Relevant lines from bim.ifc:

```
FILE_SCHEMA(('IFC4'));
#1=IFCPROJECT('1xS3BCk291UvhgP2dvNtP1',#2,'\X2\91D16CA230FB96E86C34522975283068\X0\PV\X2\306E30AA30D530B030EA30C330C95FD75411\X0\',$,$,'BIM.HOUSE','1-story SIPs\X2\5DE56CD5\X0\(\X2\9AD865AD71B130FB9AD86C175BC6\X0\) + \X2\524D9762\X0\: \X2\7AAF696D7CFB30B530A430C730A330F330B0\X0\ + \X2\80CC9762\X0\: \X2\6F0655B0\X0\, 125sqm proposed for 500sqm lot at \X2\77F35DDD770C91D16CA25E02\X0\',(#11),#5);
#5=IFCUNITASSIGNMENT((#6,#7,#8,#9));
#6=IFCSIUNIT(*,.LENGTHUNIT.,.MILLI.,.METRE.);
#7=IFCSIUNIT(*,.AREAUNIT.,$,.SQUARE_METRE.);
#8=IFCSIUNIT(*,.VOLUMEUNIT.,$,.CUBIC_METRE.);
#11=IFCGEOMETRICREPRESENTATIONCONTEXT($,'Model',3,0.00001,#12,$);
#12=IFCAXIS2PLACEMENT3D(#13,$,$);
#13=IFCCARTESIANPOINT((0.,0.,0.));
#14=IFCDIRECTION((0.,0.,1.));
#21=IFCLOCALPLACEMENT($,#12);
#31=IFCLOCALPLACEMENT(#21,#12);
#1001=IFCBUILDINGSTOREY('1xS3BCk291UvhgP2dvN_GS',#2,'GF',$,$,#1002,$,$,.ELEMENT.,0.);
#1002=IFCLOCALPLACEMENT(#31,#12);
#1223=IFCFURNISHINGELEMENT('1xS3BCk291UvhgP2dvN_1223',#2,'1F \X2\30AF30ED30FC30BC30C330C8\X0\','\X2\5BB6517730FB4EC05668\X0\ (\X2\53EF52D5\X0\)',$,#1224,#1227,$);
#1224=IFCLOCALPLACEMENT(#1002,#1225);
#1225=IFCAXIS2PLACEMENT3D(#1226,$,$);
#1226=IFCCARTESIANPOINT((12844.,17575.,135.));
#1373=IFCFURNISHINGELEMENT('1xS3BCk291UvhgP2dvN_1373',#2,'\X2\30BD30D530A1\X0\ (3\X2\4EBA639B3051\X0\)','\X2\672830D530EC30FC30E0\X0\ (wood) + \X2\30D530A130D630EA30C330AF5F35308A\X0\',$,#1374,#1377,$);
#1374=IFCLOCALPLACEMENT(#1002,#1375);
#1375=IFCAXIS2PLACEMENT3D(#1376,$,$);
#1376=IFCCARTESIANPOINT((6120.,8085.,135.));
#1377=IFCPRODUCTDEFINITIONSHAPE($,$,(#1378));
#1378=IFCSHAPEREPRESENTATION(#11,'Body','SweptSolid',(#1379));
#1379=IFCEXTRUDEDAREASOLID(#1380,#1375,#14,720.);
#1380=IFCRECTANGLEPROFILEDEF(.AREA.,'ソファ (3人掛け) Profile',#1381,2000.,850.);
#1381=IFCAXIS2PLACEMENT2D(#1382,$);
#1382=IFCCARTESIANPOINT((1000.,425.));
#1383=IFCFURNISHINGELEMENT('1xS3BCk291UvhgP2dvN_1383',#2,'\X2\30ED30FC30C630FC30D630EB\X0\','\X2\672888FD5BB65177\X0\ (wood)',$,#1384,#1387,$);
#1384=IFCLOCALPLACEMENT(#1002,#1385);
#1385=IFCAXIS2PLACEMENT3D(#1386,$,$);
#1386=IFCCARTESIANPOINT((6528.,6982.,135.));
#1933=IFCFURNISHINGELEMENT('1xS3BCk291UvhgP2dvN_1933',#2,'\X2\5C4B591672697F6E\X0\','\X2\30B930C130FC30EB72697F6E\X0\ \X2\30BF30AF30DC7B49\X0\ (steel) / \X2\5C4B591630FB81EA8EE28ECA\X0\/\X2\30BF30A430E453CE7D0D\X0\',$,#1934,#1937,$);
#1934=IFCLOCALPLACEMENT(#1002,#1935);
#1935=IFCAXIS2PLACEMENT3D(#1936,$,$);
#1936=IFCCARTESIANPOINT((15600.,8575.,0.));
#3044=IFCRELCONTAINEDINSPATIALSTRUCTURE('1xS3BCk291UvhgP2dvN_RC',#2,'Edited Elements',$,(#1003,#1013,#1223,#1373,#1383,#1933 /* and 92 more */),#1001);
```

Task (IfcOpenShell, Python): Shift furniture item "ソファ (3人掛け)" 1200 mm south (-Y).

```python
import ifcopenshell
import ifcopenshell.api.geometry
import ifcopenshell.util.placement

model = ifcopenshell.open("bim.ifc")

item = model.by_guid("1xS3BCk291UvhgP2dvN_1373")
matrix = ifcopenshell.util.placement.get_local_placement(item.ObjectPlacement)
matrix[1, 3] -= 1200.0
ifcopenshell.api.geometry.edit_object_placement(model, product=item, matrix=matrix, is_si=False)

print(ifcopenshell.util.placement.get_local_placement(item.ObjectPlacement).round(3) + 0.0)

model.write("bim_v2.ifc")
```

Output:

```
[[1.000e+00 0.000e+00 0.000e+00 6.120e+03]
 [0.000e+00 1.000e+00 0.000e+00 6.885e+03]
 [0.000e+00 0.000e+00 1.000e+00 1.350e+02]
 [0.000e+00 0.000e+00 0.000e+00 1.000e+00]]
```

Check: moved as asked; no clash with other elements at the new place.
